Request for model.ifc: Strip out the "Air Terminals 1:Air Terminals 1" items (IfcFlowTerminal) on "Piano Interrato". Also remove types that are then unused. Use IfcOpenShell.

First a look at what the model holds.

```python
import ifcopenshell
import ifcopenshell.util.element

model = ifcopenshell.open("model.ifc")
print(model.schema)
storey = next(s for s in model.by_type("IfcBuildingStorey") if s.Name == "Piano Interrato")
terminals = [e for e in ifcopenshell.util.element.get_decomposition(storey) if e.is_a("IfcFlowTerminal")]
seen = {}
for e in terminals:
    element_type = ifcopenshell.util.element.get_type(e)
    name = element_type.Name if element_type not in (None, e) else None
    seen[name] = seen.get(name, 0) + 1
for name, count in sorted(seen.items(), key=str):
    print(count, "x", name)
```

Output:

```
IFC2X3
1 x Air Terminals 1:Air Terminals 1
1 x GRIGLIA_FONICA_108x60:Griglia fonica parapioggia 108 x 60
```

```python
import ifcopenshell
import ifcopenshell.api.root
import ifcopenshell.util.element

model = ifcopenshell.open("model.ifc")

storey = next(s for s in model.by_type("IfcBuildingStorey") if s.Name == "Piano Interrato")
terminals = [e for e in ifcopenshell.util.element.get_decomposition(storey) if e.is_a("IfcFlowTerminal")]
targets = [e for e in terminals if (t := ifcopenshell.util.element.get_type(e)) not in (None, e) and t.Name == "Air Terminals 1:Air Terminals 1"]
types = {ifcopenshell.util.element.get_type(e) for e in targets} - {None, *targets}

for e in targets:
    ifcopenshell.api.root.remove_product(model, product=e)
print(len(targets), "removed")

unused = [t for t in types if not ifcopenshell.util.element.get_types(t)]
for t in unused:
    ifcopenshell.api.root.remove_product(model, product=t)
print(len(unused), "unused types removed")

model.write("model-out.ifc")
```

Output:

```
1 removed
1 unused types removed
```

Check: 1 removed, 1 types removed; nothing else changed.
